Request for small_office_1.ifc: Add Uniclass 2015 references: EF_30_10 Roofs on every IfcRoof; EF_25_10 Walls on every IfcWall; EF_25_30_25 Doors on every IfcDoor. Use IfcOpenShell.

First a look at what the model holds.

```python
import ifcopenshell

model = ifcopenshell.open("small_office_1.ifc")
print(model.schema)
print("classifications:", [c.Name for c in model.by_type("IfcClassification")])
for ifc_class in ("IfcDoor", "IfcRoof", "IfcStair", "IfcWall", "IfcWindow"):
    print(ifc_class, len(model.by_type(ifc_class)))
```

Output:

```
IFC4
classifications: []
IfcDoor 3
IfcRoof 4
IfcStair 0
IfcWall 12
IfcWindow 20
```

```python
import ifcopenshell
import ifcopenshell.api.classification

model = ifcopenshell.open("small_office_1.ifc")

system = ifcopenshell.api.classification.add_classification(model, classification="Uniclass 2015")

codes = {
    "IfcRoof": ("EF_30_10", "Roofs"),
    "IfcWall": ("EF_25_10", "Walls"),
    "IfcDoor": ("EF_25_30_25", "Doors"),
}
for ifc_class, (code, name) in codes.items():
    products = model.by_type(ifc_class)
    ifcopenshell.api.classification.add_reference(
        model, products=products, classification=system, identification=code, name=name
    )
    print(code, len(products))

model.write("small_office_1_v2.ifc")
```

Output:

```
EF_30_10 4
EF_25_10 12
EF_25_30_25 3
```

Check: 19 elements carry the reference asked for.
